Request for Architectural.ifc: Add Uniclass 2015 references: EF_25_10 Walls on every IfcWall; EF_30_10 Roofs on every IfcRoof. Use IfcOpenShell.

First a look at what the model holds.

```python
import ifcopenshell

model = ifcopenshell.open("Architectural.ifc")
print(model.schema)
print("classifications:", [c.Name for c in model.by_type("IfcClassification")])
for ifc_class in ("IfcDoor", "IfcRoof", "IfcStair", "IfcWall", "IfcWindow"):
    print(ifc_class, len(model.by_type(ifc_class)))
```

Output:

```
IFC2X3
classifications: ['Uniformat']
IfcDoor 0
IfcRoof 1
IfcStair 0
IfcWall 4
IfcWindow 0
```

```python
import ifcopenshell
import ifcopenshell.api.classification

model = ifcopenshell.open("Architectural.ifc")

# IFC2X3 requires Source and Edition and has no link from the project to the system.
system = model.create_entity("IfcClassification", Source="NBS", Edition="2015", Name="Uniclass 2015")

codes = {
    "IfcWall": ("EF_25_10", "Walls"),
    "IfcRoof": ("EF_30_10", "Roofs"),
}
for ifc_class, (code, name) in codes.items():
    products = model.by_type(ifc_class)
    ifcopenshell.api.classification.add_reference(
        model, products=products, classification=system, identification=code, name=name
    )
    print(code, len(products))

model.write("Architectural_rev.ifc")
```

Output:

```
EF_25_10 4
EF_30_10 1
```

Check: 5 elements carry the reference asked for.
